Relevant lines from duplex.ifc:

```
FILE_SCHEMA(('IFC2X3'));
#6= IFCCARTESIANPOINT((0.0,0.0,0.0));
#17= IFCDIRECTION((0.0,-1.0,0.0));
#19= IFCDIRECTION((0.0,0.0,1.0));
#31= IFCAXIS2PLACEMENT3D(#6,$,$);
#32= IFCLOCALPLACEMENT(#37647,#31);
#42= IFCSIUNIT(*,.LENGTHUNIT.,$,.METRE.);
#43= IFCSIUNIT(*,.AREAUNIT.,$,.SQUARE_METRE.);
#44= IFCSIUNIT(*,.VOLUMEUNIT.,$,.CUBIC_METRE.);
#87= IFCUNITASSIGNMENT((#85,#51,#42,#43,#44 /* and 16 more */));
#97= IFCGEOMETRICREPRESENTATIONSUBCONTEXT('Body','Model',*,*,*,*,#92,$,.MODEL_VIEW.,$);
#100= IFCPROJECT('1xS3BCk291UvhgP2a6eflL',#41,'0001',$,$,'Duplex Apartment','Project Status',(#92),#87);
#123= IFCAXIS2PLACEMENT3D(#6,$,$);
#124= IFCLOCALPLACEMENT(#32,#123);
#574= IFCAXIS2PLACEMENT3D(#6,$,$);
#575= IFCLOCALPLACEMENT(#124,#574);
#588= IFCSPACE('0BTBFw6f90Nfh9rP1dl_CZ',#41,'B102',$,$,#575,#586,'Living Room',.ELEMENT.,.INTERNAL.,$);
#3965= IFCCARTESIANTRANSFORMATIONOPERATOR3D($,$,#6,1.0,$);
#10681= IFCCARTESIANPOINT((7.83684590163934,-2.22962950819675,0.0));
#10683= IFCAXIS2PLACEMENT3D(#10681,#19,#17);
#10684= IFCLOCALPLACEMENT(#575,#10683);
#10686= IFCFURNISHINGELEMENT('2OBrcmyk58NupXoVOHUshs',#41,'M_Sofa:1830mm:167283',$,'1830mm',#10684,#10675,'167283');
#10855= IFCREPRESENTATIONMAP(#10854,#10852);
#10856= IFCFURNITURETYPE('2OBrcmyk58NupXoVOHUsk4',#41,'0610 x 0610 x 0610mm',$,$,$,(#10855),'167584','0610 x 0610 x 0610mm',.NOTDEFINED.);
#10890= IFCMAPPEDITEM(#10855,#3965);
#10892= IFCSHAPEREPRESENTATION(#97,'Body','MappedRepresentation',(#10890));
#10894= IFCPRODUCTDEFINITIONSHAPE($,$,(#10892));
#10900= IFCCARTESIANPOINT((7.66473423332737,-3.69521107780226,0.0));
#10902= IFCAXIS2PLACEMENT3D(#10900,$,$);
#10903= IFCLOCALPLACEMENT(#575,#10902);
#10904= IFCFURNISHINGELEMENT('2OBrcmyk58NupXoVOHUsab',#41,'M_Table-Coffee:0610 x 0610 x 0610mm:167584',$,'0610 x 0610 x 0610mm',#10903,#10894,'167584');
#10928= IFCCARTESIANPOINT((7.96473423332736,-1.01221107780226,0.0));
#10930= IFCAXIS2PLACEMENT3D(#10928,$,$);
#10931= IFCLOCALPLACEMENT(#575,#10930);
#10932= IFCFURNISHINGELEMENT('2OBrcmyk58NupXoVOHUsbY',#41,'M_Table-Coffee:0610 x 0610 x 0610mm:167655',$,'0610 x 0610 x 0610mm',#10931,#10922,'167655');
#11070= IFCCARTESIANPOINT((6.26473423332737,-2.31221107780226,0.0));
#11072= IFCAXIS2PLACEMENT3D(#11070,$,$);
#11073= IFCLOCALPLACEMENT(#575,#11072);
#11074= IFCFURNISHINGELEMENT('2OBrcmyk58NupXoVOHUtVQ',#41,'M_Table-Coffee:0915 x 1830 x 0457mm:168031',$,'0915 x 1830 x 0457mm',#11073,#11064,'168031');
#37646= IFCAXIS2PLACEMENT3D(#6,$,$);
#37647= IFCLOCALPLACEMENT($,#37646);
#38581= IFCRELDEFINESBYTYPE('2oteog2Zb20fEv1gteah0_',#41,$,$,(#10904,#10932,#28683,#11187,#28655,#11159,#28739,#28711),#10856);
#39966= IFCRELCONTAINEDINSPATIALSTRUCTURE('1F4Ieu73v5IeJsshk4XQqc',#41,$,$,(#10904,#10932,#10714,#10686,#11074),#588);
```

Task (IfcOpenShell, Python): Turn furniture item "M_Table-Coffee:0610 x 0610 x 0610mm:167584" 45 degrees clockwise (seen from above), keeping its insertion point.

```python
import ifcopenshell
import ifcopenshell.api.geometry
import ifcopenshell.util.placement

model = ifcopenshell.open("duplex.ifc")

item = model.by_guid("2OBrcmyk58NupXoVOHUsab")
matrix = ifcopenshell.util.placement.get_local_placement(item.ObjectPlacement)
matrix = matrix @ ifcopenshell.util.placement.rotation(-45, "Z")
ifcopenshell.api.geometry.edit_object_placement(model, product=item, matrix=matrix, is_si=False)

print(ifcopenshell.util.placement.get_local_placement(item.ObjectPlacement).round(3) + 0.0)

model.write("duplex_v2.ifc")
```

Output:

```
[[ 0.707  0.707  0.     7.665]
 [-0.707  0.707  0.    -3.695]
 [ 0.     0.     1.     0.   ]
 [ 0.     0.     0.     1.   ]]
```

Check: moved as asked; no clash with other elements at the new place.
